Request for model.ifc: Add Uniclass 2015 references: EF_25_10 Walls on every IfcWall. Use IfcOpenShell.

First a look at what the model holds.

```python
import ifcopenshell

model = ifcopenshell.open("model.ifc")
print(model.schema)
print("classifications:", [c.Name for c in model.by_type("IfcClassification")])
for ifc_class in ("IfcDoor", "IfcRoof", "IfcStair", "IfcWall", "IfcWindow"):
    print(ifc_class, len(model.by_type(ifc_class)))
```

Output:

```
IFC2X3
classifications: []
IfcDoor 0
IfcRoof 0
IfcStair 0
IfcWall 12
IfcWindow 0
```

```python
import ifcopenshell
import ifcopenshell.api.classification

model = ifcopenshell.open("model.ifc")

# IFC2X3 requires Source and Edition and has no link from the project to the system.
system = model.create_entity("IfcClassification", Source="NBS", Edition="2015", Name="Uniclass 2015")

codes = {
    "IfcWall": ("EF_25_10", "Walls"),
}
for ifc_class, (code, name) in codes.items():
    products = model.by_type(ifc_class)
    ifcopenshell.api.classification.add_reference(
        model, products=products, classification=system, identification=code, name=name
    )
    print(code, len(products))

model.write("model_updated.ifc")
```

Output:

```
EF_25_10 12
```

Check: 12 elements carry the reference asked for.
